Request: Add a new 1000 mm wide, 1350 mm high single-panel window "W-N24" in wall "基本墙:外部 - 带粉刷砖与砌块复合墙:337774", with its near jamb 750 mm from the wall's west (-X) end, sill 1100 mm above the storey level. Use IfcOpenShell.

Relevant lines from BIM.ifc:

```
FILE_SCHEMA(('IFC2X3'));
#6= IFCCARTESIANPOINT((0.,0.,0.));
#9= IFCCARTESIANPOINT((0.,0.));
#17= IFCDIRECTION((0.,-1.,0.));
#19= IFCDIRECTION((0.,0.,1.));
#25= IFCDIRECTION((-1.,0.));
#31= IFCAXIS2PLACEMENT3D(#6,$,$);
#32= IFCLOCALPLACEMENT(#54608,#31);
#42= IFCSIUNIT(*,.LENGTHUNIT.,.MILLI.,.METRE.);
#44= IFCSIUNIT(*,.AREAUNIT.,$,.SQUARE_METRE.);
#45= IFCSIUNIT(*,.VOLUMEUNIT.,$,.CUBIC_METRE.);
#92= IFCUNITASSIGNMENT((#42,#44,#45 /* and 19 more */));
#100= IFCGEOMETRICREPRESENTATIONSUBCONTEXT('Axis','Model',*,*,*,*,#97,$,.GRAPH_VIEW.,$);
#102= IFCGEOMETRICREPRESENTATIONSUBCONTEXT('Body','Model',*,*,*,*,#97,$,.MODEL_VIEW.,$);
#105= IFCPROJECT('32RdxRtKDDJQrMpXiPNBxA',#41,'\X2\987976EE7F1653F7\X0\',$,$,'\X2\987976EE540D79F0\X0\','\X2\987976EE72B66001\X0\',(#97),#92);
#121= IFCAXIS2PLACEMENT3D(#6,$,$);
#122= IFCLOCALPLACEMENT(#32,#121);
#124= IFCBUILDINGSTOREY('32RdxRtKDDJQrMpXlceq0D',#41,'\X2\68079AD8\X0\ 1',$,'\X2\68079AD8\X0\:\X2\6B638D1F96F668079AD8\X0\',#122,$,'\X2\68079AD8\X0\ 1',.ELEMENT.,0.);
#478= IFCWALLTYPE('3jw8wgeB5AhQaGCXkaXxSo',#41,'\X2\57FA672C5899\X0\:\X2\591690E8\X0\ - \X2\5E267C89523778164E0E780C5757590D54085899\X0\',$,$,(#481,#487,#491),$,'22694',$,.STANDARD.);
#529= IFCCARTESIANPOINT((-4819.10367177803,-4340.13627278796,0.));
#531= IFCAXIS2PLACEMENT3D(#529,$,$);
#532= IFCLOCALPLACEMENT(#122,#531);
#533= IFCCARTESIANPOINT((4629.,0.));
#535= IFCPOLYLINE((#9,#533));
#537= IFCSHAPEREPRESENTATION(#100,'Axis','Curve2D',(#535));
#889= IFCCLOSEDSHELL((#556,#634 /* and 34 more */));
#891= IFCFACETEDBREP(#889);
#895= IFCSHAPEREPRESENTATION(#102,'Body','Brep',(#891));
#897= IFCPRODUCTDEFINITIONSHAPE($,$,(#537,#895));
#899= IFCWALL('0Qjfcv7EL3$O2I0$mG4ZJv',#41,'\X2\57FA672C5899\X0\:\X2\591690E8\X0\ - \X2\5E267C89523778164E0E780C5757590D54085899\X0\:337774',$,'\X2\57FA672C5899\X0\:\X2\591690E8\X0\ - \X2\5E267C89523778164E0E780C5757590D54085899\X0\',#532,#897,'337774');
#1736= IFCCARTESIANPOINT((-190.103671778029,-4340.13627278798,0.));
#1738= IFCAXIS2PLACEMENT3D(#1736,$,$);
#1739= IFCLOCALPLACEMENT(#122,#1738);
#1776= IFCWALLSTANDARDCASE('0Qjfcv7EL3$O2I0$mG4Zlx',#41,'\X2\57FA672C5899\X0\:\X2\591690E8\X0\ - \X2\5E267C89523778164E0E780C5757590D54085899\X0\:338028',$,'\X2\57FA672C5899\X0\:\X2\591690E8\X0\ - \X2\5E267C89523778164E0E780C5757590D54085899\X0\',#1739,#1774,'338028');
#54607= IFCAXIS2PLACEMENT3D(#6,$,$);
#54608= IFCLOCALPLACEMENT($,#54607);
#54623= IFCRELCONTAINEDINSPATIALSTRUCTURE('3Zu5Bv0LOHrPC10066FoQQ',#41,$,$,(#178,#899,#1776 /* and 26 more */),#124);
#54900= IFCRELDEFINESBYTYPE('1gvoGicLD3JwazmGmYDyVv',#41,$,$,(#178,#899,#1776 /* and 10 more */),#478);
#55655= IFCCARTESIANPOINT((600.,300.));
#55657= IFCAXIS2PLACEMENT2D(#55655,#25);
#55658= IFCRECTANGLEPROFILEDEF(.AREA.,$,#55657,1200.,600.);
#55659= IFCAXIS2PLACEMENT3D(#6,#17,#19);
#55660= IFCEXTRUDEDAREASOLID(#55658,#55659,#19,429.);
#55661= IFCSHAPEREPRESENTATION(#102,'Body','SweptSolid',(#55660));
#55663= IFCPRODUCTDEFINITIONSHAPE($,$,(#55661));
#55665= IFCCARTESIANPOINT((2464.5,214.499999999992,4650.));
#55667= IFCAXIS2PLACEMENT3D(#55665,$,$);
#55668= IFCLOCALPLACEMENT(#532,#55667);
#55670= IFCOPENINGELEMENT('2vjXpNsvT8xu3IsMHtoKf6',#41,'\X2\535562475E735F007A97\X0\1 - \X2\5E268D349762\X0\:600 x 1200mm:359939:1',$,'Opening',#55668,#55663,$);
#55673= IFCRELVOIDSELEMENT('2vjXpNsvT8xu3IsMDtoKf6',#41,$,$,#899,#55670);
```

```python
import numpy as np
import ifcopenshell
import ifcopenshell.api.feature
import ifcopenshell.api.geometry
import ifcopenshell.api.root
import ifcopenshell.api.spatial
import ifcopenshell.api.type
import ifcopenshell.geom
import ifcopenshell.util.element
import ifcopenshell.util.placement
import ifcopenshell.util.representation
import ifcopenshell.util.shape
import ifcopenshell.util.unit

model = ifcopenshell.open("BIM.ifc")
unit_scale = ifcopenshell.util.unit.calculate_unit_scale(model)
settings = ifcopenshell.geom.settings()


def volume(element):
    """Net volume in cubic metres, openings subtracted."""
    shape = ifcopenshell.geom.create_shape(settings, element)
    return ifcopenshell.util.shape.get_volume(shape.geometry)


wall = model.by_id(899)
storey = ifcopenshell.util.element.get_container(wall, ifc_class="IfcBuildingStorey")
context = ifcopenshell.util.representation.get_context(model, "Model", "Body", "MODEL_VIEW")
before = volume(wall)

width, height, from_end, sill = 1, 1.35, 0.75, 1.1  # metres

# The wall runs along its own X axis, and the end named is its -X end.
wall_shape = ifcopenshell.geom.create_shape(settings, wall)
x, y, z = ifcopenshell.util.shape.get_vertices(wall_shape.geometry).T
start = x.min() + from_end
face, thickness = float(y.min()), float(y.max() - y.min())
wall_matrix = ifcopenshell.util.placement.get_local_placement(wall.ObjectPlacement)
level = ifcopenshell.util.placement.get_local_placement(storey.ObjectPlacement)[2, 3]


def in_wall(x, y):
    """Placement at x, y metres in the wall's axes, at sill height."""
    matrix = wall_matrix.copy()
    matrix[:, 3] = wall_matrix @ np.array([x / unit_scale, y / unit_scale, 0.0, 1.0])
    matrix[2, 3] = level + sill / unit_scale
    return matrix


# Opening: a box that overshoots both wall faces by 50 mm.
opening = ifcopenshell.api.root.create_entity(model, ifc_class="IfcOpeningElement")
box = ifcopenshell.api.geometry.add_wall_representation(
    model, context=context, length=width, height=height, thickness=thickness + 0.1
)
ifcopenshell.api.geometry.assign_representation(model, product=opening, representation=box)
ifcopenshell.api.geometry.edit_object_placement(model, product=opening, matrix=in_wall(start, face - 0.05), is_si=False)
ifcopenshell.api.feature.add_feature(model, feature=opening, element=wall)

window = ifcopenshell.api.root.create_entity(model, ifc_class="IfcWindow", name="W-N24")
window.OverallWidth, window.OverallHeight = width / unit_scale, height / unit_scale
body = ifcopenshell.api.geometry.add_window_representation(
    model,
    context=context,
    overall_width=window.OverallWidth,
    overall_height=window.OverallHeight,
    partition_type="SINGLE_PANEL",
)
ifcopenshell.api.geometry.assign_representation(model, product=window, representation=body)
ifcopenshell.api.spatial.assign_container(model, products=[window], relating_structure=storey)
fills = ifcopenshell.api.feature.add_filling(model, opening=opening, element=window)
fills.OwnerHistory = window.OwnerHistory  # required in IFC2X3

# IFC2X3 keeps the operation on the window style.
style = ifcopenshell.api.root.create_entity(model, ifc_class="IfcWindowStyle", name="W-N24")
style.OperationType, style.ConstructionType = "SINGLE_PANEL", "NOTDEFINED"
style.ParameterTakesPrecedence = style.Sizeable = False
ifcopenshell.api.type.assign_type(model, related_objects=[window], relating_type=style)

# Centre the window in the wall's thickness.
ifcopenshell.api.geometry.edit_object_placement(model, product=window, matrix=in_wall(start, face), is_si=False)
window_shape = ifcopenshell.geom.create_shape(settings, window)
depth = ifcopenshell.util.shape.get_vertices(window_shape.geometry)[:, 1]
offset = face + thickness / 2 - (depth.min() + depth.max()) / 2
ifcopenshell.api.geometry.edit_object_placement(model, product=window, matrix=in_wall(start, offset), is_si=False)

after = volume(wall)

print(f"wall volume {before:.3f} -> {after:.3f} m3")

model.write("BIM_edited.ifc")
```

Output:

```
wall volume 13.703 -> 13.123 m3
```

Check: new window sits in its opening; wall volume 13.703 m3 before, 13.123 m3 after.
